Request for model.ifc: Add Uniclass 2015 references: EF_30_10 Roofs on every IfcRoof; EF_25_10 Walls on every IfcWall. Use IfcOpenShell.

First a look at what the model holds.

```python
import ifcopenshell

model = ifcopenshell.open("model.ifc")
print(model.schema)
print("classifications:", [c.Name for c in model.by_type("IfcClassification")])
for ifc_class in ("IfcDoor", "IfcRoof", "IfcStair", "IfcWall", "IfcWindow"):
    print(ifc_class, len(model.by_type(ifc_class)))
```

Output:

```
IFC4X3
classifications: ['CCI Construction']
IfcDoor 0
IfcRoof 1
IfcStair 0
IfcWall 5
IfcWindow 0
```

```python
import ifcopenshell
import ifcopenshell.api.classification

model = ifcopenshell.open("model.ifc")

system = ifcopenshell.api.classification.add_classification(model, classification="Uniclass 2015")

codes = {
    "IfcRoof": ("EF_30_10", "Roofs"),
    "IfcWall": ("EF_25_10", "Walls"),
}
for ifc_class, (code, name) in codes.items():
    products = model.by_type(ifc_class)
    ifcopenshell.api.classification.add_reference(
        model, products=products, classification=system, identification=code, name=name
    )
    print(code, len(products))

model.write("model_edited.ifc")
```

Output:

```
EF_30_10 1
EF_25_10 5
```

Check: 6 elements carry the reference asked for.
